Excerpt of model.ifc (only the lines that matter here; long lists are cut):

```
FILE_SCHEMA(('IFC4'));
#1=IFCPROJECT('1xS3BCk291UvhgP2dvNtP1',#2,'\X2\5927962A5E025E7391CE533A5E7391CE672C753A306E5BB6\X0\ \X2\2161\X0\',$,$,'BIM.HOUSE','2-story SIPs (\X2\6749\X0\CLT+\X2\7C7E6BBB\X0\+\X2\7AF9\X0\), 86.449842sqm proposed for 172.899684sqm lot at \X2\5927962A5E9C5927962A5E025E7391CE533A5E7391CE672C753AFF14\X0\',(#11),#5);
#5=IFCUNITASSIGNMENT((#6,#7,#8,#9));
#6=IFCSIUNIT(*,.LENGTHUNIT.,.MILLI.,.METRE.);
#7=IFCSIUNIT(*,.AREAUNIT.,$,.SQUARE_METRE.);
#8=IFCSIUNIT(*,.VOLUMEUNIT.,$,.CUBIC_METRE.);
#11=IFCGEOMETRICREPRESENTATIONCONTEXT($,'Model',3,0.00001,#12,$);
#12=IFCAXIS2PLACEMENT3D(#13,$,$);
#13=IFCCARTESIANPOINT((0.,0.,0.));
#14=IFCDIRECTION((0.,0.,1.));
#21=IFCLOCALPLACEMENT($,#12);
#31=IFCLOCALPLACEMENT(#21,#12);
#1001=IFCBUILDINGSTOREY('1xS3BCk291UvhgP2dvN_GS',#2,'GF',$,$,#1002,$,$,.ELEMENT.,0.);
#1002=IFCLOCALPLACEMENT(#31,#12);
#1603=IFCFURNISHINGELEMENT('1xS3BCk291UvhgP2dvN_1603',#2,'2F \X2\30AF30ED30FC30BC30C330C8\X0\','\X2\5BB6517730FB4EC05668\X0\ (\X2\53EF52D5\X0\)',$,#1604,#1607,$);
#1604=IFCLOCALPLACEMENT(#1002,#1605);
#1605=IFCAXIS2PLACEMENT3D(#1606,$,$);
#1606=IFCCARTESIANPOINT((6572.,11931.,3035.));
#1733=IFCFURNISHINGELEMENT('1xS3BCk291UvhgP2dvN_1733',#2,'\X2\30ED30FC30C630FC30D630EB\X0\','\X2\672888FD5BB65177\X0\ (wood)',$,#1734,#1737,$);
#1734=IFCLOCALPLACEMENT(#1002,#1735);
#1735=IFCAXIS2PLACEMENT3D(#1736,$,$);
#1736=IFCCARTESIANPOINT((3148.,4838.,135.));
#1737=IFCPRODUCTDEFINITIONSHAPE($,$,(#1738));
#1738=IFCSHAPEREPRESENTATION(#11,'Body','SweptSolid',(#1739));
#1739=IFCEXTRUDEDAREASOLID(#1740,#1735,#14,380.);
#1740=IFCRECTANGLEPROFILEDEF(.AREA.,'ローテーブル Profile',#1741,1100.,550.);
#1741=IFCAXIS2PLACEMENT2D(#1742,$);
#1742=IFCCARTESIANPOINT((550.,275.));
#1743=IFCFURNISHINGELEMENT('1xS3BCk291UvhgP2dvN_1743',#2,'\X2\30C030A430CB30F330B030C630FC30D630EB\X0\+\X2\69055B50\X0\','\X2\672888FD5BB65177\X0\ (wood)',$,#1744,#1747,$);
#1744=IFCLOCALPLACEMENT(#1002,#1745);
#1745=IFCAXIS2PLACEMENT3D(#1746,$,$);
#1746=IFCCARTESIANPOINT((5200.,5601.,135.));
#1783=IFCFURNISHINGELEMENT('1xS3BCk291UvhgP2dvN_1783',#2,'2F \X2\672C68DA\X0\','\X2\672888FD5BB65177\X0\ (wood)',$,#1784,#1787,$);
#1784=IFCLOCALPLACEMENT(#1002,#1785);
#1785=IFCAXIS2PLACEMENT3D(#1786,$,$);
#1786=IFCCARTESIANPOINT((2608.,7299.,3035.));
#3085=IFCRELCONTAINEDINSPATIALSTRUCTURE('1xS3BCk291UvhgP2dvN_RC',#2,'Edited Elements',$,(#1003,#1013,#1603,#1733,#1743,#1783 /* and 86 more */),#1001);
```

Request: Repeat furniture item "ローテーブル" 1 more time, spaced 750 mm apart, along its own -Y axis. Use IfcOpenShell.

```python
import ifcopenshell
import ifcopenshell.api.geometry
import ifcopenshell.api.root
import ifcopenshell.util.element
import ifcopenshell.util.placement

model = ifcopenshell.open("model.ifc")


def reuse_history(source, copy):
    """copy_class also copies each property set's owner history, people and application; keep the originals."""
    for rel in copy.IsDefinedBy:
        if rel.is_a("IfcRelDefinesByProperties") and (history := rel.RelatingPropertyDefinition.OwnerHistory):
            rel.RelatingPropertyDefinition.OwnerHistory = source.OwnerHistory
            ifcopenshell.util.element.remove_deep2(model, history)


source = model.by_guid("1xS3BCk291UvhgP2dvN_1733")
base = ifcopenshell.util.placement.get_local_placement(source.ObjectPlacement)
step = -base[:3, 1] * 750.0

for i in range(1, 2):
    copy = ifcopenshell.api.root.copy_class(model, product=source)
    copy.Representation = ifcopenshell.util.element.copy_deep(
        model, source.Representation, exclude=["IfcGeometricRepresentationContext", "IfcRepresentationMap"]
    )
    reuse_history(source, copy)
    matrix = base.copy()
    matrix[:3, 3] += i * step
    print("added at", matrix[:3, 3].round(3) + 0.0)
    ifcopenshell.api.geometry.edit_object_placement(model, product=copy, matrix=matrix, is_si=False)

model.write("model_rev.ifc")
```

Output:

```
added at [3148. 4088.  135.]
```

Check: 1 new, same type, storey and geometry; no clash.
